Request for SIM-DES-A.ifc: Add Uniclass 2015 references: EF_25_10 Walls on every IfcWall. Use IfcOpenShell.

First a look at what the model holds.

```python
import ifcopenshell

model = ifcopenshell.open("SIM-DES-A.ifc")
print(model.schema)
print("classifications:", [c.Name for c in model.by_type("IfcClassification")])
for ifc_class in ("IfcDoor", "IfcRoof", "IfcStair", "IfcWall", "IfcWindow"):
    print(ifc_class, len(model.by_type(ifc_class)))
```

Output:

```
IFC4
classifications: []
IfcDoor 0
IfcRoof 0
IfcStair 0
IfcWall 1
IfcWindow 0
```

```python
import ifcopenshell
import ifcopenshell.api.classification

model = ifcopenshell.open("SIM-DES-A.ifc")

system = ifcopenshell.api.classification.add_classification(model, classification="Uniclass 2015")

codes = {
    "IfcWall": ("EF_25_10", "Walls"),
}
for ifc_class, (code, name) in codes.items():
    products = model.by_type(ifc_class)
    ifcopenshell.api.classification.add_reference(
        model, products=products, classification=system, identification=code, name=name
    )
    print(code, len(products))

model.write("SIM-DES-A_v2.ifc")
```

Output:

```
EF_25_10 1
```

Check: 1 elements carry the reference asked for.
